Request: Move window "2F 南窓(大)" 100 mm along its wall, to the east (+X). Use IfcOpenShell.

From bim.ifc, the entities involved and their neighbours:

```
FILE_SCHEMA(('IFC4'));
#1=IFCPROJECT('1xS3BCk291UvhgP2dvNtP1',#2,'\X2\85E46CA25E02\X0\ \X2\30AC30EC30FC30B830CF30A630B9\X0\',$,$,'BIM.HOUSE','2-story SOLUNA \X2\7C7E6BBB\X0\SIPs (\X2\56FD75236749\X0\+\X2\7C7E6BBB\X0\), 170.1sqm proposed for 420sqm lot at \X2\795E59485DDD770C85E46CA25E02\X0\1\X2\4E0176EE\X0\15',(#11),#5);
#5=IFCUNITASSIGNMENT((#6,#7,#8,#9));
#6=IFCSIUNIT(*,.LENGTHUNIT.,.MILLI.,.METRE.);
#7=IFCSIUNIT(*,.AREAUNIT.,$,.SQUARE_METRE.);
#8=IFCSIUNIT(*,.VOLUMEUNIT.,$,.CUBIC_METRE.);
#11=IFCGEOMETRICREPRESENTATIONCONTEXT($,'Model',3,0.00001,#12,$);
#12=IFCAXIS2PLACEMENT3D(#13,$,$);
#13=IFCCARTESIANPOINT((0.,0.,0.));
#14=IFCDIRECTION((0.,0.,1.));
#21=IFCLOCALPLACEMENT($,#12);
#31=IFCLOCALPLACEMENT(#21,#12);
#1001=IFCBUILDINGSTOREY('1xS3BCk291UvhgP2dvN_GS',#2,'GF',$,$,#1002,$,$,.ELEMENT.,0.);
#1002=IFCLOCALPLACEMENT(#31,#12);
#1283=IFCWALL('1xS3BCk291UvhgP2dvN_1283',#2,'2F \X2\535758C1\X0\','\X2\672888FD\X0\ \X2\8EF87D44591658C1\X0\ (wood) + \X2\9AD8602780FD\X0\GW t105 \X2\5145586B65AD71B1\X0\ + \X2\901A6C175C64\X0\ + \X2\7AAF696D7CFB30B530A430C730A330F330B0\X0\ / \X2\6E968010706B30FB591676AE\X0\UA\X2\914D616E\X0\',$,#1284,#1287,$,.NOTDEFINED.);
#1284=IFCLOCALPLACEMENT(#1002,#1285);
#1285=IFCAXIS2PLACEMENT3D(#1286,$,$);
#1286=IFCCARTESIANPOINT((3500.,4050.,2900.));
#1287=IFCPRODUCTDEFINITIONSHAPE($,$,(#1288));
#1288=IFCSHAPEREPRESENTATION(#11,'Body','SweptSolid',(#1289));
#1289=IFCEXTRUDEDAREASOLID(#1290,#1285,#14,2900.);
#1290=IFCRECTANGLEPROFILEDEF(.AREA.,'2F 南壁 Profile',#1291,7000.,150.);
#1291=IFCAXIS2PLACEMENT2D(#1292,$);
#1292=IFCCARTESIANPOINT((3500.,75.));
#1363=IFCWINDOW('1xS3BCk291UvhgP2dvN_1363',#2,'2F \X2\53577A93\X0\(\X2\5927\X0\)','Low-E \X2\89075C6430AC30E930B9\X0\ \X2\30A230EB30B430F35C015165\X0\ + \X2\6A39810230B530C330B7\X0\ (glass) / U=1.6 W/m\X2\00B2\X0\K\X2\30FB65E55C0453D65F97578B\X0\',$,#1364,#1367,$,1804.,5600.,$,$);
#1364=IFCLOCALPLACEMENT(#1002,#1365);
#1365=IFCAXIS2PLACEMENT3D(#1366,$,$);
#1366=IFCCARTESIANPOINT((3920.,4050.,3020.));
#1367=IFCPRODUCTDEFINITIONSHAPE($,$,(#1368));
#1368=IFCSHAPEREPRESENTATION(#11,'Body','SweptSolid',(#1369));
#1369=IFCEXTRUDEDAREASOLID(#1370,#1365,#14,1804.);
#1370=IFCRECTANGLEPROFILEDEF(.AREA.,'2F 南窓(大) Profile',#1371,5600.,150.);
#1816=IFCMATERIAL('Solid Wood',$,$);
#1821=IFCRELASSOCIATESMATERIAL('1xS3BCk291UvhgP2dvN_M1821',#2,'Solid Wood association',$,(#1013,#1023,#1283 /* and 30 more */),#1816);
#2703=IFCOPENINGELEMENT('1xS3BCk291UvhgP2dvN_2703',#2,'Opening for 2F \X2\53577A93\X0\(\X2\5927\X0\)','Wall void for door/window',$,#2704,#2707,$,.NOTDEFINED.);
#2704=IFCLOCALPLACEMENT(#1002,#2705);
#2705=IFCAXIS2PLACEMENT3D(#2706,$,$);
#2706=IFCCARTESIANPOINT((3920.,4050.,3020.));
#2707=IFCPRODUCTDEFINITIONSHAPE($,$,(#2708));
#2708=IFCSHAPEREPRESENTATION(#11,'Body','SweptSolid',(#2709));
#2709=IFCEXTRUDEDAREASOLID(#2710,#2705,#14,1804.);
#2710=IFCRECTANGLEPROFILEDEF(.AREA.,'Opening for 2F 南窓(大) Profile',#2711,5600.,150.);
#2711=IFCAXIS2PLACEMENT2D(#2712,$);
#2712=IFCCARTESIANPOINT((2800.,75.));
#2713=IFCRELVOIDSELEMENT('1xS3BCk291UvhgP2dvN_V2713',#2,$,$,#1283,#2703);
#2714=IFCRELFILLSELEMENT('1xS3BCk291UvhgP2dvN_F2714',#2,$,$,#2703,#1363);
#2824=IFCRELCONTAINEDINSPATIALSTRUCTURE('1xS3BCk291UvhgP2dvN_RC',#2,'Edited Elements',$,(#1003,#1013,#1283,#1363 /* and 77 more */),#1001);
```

```python
import ifcopenshell
import ifcopenshell.api.geometry
import ifcopenshell.util.placement
import ifcopenshell.util.unit

model = ifcopenshell.open("bim.ifc")
unit_scale = ifcopenshell.util.unit.calculate_unit_scale(model)

window = model.by_guid("1xS3BCk291UvhgP2dvN_1363")
opening = window.FillsVoids[0].RelatingOpeningElement
wall = opening.VoidsElements[0].RelatingBuildingElement

wall_matrix = ifcopenshell.util.placement.get_local_placement(wall.ObjectPlacement)
shift = wall_matrix[:3, 0] * 0.1 / unit_scale
before = ifcopenshell.util.placement.get_local_placement(window.ObjectPlacement)[:3, 3].copy()

# The window is not placed relative to its opening, so move both.
for product in (opening, window):
    matrix = ifcopenshell.util.placement.get_local_placement(product.ObjectPlacement)
    matrix[:3, 3] += shift
    ifcopenshell.api.geometry.edit_object_placement(model, product=product, matrix=matrix, is_si=False)

after = ifcopenshell.util.placement.get_local_placement(window.ObjectPlacement)[:3, 3]
print("window moved by", (after - before).round(3) + 0.0)

model.write("bim_rev.ifc")
```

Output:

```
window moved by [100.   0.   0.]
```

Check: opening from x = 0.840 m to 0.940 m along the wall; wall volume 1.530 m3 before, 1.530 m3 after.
